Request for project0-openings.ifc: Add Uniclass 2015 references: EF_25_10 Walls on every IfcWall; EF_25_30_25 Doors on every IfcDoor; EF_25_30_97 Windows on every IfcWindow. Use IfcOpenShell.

First a look at what the model holds.

```python
import ifcopenshell

model = ifcopenshell.open("project0-openings.ifc")
print(model.schema)
print("classifications:", [c.Name for c in model.by_type("IfcClassification")])
for ifc_class in ("IfcDoor", "IfcRoof", "IfcStair", "IfcWall", "IfcWindow"):
    print(ifc_class, len(model.by_type(ifc_class)))
```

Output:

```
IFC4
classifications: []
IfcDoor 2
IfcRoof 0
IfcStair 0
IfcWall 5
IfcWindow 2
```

```python
import ifcopenshell
import ifcopenshell.api.classification

model = ifcopenshell.open("project0-openings.ifc")

system = ifcopenshell.api.classification.add_classification(model, classification="Uniclass 2015")

codes = {
    "IfcWall": ("EF_25_10", "Walls"),
    "IfcDoor": ("EF_25_30_25", "Doors"),
    "IfcWindow": ("EF_25_30_97", "Windows"),
}
for ifc_class, (code, name) in codes.items():
    products = model.by_type(ifc_class)
    ifcopenshell.api.classification.add_reference(
        model, products=products, classification=system, identification=code, name=name
    )
    print(code, len(products))

model.write("project0-openings_rev.ifc")
```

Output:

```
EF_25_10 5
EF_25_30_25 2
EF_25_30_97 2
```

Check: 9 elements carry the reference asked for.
